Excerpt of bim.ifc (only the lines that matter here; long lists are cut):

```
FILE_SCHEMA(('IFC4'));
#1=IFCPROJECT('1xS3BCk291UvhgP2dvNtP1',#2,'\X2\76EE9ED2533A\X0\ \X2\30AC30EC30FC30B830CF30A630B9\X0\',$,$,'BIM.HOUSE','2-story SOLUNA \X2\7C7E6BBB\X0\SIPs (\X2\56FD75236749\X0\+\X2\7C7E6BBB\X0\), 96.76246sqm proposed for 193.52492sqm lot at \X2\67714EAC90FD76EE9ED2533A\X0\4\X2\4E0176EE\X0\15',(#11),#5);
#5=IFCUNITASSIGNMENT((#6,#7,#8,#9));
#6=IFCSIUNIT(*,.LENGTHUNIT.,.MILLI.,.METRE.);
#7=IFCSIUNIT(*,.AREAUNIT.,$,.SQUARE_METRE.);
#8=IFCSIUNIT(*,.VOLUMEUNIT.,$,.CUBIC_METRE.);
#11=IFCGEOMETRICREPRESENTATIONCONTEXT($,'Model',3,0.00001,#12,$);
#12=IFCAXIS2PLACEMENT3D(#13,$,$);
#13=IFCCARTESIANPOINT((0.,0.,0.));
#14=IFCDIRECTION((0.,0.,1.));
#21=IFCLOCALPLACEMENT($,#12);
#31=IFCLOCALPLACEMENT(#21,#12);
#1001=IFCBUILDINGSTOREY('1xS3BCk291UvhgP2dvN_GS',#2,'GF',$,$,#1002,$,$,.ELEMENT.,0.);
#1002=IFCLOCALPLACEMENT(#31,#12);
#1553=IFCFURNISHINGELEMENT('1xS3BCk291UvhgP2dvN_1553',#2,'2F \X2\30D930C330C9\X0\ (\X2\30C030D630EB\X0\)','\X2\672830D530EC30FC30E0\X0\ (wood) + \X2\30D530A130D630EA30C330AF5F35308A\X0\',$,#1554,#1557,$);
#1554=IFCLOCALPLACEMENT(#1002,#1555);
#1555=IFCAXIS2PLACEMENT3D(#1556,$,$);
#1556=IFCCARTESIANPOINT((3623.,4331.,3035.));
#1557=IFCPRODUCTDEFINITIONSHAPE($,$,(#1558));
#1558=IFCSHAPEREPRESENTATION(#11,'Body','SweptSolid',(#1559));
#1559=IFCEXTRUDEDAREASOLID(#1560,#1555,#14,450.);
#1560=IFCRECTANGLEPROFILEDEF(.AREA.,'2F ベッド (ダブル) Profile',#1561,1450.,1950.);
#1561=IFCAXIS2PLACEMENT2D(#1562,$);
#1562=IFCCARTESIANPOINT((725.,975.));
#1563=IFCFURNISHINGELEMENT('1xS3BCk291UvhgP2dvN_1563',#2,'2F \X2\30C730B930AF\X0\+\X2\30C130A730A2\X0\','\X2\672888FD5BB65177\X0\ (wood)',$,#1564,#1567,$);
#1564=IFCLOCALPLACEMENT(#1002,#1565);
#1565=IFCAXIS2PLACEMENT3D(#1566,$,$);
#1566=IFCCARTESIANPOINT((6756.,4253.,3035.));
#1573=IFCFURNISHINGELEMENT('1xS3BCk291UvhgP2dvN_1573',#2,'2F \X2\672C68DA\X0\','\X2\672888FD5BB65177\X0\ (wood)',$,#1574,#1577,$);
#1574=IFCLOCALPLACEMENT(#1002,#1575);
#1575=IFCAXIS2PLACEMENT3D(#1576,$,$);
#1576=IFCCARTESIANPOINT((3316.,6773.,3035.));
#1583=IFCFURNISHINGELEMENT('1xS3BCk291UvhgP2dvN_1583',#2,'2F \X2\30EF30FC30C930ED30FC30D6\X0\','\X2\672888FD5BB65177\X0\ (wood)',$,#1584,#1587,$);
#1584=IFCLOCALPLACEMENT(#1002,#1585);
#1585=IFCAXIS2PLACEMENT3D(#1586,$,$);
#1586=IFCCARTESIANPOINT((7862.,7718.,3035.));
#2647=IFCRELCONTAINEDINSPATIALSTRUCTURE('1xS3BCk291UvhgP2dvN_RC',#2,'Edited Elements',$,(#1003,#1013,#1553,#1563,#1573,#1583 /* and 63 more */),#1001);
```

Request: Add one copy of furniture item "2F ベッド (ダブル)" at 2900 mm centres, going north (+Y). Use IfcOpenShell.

```python
import numpy as np
import ifcopenshell
import ifcopenshell.api.geometry
import ifcopenshell.api.root
import ifcopenshell.util.element
import ifcopenshell.util.placement
import ifcopenshell.util.unit

model = ifcopenshell.open("bim.ifc")
unit_scale = ifcopenshell.util.unit.calculate_unit_scale(model)


def reuse_history(source, copy):
    """copy_class also copies each property set's owner history, people and application; keep the originals."""
    for rel in copy.IsDefinedBy:
        if rel.is_a("IfcRelDefinesByProperties") and (history := rel.RelatingPropertyDefinition.OwnerHistory):
            rel.RelatingPropertyDefinition.OwnerHistory = source.OwnerHistory
            ifcopenshell.util.element.remove_deep2(model, history)


source = model.by_guid("1xS3BCk291UvhgP2dvN_1553")
base = ifcopenshell.util.placement.get_local_placement(source.ObjectPlacement)
step = np.array([0.0, 1.0, 0.0]) * 2.9 / unit_scale

for i in range(1, 2):
    copy = ifcopenshell.api.root.copy_class(model, product=source)
    copy.Representation = ifcopenshell.util.element.copy_deep(
        model, source.Representation, exclude=["IfcGeometricRepresentationContext", "IfcRepresentationMap"]
    )
    reuse_history(source, copy)
    matrix = base.copy()
    matrix[:3, 3] += i * step
    print("added at", matrix[:3, 3].round(3) + 0.0)
    ifcopenshell.api.geometry.edit_object_placement(model, product=copy, matrix=matrix, is_si=False)

model.write("bim_rev.ifc")
```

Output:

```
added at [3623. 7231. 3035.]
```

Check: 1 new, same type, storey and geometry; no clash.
